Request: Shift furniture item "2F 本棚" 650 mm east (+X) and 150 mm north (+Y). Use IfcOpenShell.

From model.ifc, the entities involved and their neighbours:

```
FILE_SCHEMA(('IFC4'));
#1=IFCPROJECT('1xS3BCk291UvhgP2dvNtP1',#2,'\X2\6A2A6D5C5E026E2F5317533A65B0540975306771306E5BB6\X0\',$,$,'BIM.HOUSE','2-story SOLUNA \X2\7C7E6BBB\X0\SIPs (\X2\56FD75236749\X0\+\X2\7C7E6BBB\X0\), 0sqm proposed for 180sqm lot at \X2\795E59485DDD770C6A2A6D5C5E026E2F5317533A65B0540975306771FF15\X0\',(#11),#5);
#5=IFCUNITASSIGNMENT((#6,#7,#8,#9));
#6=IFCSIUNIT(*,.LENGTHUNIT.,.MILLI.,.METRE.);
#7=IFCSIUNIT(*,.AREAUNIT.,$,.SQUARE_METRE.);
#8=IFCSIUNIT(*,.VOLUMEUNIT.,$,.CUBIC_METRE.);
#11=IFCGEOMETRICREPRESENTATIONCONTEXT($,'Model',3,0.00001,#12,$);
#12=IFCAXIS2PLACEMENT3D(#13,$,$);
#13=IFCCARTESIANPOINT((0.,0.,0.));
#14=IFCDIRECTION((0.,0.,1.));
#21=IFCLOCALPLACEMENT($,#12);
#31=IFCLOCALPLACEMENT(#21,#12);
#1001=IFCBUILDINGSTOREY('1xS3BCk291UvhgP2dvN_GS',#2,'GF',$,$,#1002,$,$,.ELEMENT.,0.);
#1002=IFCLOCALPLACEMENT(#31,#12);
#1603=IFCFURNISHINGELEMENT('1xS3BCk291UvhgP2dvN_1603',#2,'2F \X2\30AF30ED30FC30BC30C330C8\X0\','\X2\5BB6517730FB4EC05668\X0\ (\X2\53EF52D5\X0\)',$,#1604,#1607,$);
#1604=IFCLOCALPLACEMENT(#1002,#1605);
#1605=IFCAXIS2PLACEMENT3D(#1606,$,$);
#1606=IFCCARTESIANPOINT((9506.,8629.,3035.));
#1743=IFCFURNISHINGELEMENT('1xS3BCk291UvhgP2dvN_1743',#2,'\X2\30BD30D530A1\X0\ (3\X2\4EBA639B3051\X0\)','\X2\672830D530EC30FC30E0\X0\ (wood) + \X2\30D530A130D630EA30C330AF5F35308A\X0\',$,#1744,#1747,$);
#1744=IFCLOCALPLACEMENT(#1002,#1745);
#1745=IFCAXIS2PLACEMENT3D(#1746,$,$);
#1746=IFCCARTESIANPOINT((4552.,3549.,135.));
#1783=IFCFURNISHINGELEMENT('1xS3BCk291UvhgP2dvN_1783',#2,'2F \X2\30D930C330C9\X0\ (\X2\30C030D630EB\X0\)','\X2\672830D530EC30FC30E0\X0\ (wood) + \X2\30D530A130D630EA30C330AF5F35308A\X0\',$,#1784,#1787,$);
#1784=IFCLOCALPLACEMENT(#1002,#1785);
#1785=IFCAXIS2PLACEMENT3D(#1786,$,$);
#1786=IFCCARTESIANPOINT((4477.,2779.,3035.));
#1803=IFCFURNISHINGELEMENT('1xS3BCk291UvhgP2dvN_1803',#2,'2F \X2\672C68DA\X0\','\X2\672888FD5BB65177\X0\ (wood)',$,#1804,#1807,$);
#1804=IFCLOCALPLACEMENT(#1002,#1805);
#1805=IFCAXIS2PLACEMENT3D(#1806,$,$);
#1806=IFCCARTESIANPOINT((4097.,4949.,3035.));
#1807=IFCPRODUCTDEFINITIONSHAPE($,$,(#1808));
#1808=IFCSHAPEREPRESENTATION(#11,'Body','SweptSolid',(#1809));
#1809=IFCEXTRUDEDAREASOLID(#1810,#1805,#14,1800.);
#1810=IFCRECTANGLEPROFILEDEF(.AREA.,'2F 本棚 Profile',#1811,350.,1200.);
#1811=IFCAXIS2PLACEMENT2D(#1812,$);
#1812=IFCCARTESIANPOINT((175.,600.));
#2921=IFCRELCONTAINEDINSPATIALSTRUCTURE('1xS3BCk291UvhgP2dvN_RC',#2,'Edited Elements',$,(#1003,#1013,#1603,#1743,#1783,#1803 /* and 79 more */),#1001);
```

```python
import ifcopenshell
import ifcopenshell.api.geometry
import ifcopenshell.util.placement
import ifcopenshell.util.unit

model = ifcopenshell.open("model.ifc")
unit_scale = ifcopenshell.util.unit.calculate_unit_scale(model)

item = model.by_id(1803)
matrix = ifcopenshell.util.placement.get_local_placement(item.ObjectPlacement)
matrix[0, 3] += 0.65 / unit_scale
matrix[1, 3] += 0.15 / unit_scale
ifcopenshell.api.geometry.edit_object_placement(model, product=item, matrix=matrix, is_si=False)

print(ifcopenshell.util.placement.get_local_placement(item.ObjectPlacement).round(3) + 0.0)

model.write("model_rev.ifc")
```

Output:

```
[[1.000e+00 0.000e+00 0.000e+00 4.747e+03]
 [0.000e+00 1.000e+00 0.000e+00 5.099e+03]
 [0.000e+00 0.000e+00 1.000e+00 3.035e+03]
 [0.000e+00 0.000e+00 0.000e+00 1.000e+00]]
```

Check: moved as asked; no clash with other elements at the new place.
